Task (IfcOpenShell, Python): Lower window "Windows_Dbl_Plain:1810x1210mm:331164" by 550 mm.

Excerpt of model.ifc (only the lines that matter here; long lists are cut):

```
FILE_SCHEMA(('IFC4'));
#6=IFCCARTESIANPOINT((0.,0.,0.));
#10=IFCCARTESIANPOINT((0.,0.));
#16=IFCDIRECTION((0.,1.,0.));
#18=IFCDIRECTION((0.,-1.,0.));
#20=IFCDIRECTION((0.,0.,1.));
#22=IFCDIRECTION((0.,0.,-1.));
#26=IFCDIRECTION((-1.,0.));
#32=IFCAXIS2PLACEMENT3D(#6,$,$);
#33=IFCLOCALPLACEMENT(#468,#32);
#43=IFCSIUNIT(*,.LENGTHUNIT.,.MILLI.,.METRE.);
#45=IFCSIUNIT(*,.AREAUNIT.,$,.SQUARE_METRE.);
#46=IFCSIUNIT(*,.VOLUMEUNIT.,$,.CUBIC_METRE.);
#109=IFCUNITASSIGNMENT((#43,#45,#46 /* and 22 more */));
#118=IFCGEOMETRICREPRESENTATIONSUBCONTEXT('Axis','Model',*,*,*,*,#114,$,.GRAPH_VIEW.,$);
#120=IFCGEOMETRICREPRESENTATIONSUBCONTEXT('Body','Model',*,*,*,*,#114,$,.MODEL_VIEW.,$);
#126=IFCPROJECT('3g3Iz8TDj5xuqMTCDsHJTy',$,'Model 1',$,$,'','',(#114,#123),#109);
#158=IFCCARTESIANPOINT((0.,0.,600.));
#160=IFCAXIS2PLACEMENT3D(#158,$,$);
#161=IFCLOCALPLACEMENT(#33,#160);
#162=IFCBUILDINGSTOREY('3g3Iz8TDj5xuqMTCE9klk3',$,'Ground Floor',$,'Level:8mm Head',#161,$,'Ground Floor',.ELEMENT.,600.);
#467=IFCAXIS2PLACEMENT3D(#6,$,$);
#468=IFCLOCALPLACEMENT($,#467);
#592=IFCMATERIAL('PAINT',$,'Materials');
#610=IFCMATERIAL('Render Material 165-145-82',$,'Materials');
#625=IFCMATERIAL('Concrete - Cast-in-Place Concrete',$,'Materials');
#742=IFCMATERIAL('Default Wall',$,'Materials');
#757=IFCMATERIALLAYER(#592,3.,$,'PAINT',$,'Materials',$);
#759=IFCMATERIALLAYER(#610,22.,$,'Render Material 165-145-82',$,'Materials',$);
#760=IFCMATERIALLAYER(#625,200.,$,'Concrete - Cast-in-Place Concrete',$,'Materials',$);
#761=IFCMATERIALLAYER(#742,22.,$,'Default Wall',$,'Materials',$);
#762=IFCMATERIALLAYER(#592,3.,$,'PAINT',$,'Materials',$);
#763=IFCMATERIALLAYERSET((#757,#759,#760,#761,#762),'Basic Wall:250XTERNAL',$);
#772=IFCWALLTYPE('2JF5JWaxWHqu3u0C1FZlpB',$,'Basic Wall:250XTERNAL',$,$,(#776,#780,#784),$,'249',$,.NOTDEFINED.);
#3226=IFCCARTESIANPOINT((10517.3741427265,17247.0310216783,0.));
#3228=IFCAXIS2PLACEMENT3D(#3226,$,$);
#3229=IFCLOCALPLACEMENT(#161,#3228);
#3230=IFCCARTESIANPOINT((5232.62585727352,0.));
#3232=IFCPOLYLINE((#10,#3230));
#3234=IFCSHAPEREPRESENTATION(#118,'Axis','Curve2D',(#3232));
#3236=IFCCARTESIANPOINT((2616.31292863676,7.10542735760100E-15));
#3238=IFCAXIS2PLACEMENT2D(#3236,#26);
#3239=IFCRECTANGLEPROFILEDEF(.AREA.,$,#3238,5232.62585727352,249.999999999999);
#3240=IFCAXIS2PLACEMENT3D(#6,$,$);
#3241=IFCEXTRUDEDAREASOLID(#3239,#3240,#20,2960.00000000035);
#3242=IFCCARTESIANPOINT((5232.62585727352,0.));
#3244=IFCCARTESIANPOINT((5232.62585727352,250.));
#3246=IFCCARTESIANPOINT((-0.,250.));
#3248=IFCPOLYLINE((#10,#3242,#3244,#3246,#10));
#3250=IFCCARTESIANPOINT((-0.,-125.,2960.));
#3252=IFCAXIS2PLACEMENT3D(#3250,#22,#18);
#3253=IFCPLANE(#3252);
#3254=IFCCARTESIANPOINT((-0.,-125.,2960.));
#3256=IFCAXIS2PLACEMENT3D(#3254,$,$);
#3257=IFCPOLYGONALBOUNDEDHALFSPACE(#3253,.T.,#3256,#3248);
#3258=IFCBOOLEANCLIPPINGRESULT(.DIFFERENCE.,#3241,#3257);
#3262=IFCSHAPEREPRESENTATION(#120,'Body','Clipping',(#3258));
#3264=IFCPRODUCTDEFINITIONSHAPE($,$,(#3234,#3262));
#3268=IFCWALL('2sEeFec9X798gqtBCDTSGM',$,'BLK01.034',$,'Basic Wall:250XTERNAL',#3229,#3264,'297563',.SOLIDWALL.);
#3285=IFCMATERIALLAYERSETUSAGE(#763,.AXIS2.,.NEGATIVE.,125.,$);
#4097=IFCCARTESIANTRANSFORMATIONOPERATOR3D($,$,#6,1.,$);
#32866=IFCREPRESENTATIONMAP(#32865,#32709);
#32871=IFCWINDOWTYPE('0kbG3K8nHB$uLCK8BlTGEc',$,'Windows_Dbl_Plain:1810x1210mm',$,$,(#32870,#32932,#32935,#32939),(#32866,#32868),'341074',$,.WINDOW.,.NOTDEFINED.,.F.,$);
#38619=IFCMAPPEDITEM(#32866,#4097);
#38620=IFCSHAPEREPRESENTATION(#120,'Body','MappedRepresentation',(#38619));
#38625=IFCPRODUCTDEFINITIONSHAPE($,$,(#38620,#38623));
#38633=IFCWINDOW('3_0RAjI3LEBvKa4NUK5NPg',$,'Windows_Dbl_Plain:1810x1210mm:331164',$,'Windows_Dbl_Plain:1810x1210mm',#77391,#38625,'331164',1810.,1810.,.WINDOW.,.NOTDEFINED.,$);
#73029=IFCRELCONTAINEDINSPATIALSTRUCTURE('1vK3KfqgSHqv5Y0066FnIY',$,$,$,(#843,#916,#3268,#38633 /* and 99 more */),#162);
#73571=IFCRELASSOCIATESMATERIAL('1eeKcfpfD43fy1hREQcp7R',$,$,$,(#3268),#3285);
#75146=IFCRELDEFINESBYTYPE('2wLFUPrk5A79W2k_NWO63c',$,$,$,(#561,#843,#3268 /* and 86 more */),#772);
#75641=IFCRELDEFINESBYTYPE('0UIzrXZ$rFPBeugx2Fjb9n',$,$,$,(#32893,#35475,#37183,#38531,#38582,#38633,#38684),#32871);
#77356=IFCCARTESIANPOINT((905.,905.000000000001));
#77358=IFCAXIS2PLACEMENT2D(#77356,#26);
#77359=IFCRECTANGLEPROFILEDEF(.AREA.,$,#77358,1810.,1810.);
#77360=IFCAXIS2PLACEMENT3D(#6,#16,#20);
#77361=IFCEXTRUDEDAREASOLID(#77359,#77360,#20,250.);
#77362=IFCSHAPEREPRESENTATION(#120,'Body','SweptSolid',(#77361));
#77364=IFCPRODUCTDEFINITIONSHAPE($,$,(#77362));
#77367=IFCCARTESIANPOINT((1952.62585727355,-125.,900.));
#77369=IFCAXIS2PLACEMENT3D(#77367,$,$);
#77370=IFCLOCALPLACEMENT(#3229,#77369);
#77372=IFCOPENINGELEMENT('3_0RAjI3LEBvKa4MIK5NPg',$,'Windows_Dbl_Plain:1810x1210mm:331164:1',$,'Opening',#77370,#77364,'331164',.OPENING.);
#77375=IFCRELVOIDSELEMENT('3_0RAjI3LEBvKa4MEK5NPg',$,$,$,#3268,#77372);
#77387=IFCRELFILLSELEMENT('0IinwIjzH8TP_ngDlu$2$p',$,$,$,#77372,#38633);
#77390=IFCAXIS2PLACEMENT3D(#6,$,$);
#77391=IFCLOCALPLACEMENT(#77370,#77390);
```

```python
import numpy as np
import ifcopenshell
import ifcopenshell.api.geometry
import ifcopenshell.util.placement
import ifcopenshell.util.unit

model = ifcopenshell.open("model.ifc")
unit_scale = ifcopenshell.util.unit.calculate_unit_scale(model)

window = model.by_id(38633)
opening = window.FillsVoids[0].RelatingOpeningElement
dz = -550.0

shift = np.array([0.0, 0.0, dz])
# The window is placed relative to its opening, so it follows when the opening moves.
matrix = ifcopenshell.util.placement.get_local_placement(opening.ObjectPlacement)
matrix[:3, 3] += shift
ifcopenshell.api.geometry.edit_object_placement(
    model, product=opening, matrix=matrix, is_si=False, should_transform_children=True
)

print(f"moved by {dz * unit_scale:+.3f} m")

model.write("model_updated.ifc")
```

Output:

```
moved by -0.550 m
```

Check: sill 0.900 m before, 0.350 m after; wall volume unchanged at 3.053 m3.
